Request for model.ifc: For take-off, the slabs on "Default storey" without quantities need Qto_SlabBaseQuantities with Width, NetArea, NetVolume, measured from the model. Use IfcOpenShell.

First a look at what the model holds.

```python
import ifcopenshell
import ifcopenshell.util.element
import ifcopenshell.util.unit

model = ifcopenshell.open("model.ifc")
print(model.schema)
for unit_type in ("LENGTHUNIT", "AREAUNIT", "VOLUMEUNIT"):
    print(unit_type, ifcopenshell.util.unit.calculate_unit_scale(model, unit_type))
storey = next(s for s in model.by_type("IfcBuildingStorey") if s.Name == "Default storey")
slabs = [e for e in ifcopenshell.util.element.get_decomposition(storey) if e.is_a("IfcSlab")]
for e in sorted(slabs, key=lambda e: e.id()):
    print(e.id(), e.is_a(), e.Name, list(ifcopenshell.util.element.get_psets(e, qtos_only=True)), sep=" | ")
```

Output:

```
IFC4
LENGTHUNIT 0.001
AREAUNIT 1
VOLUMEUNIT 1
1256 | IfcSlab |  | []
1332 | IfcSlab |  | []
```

```python
import ifcopenshell
import ifcopenshell.api.pset
import ifcopenshell.geom
import ifcopenshell.util.element
import ifcopenshell.util.shape
import ifcopenshell.util.unit

model = ifcopenshell.open("model.ifc")
unit_scale = ifcopenshell.util.unit.calculate_unit_scale(model)
area_scale = ifcopenshell.util.unit.calculate_unit_scale(model, "AREAUNIT")
volume_scale = ifcopenshell.util.unit.calculate_unit_scale(model, "VOLUMEUNIT")
settings = ifcopenshell.geom.settings()

storey = next(s for s in model.by_type("IfcBuildingStorey") if s.Name == "Default storey")
slabs = [e for e in ifcopenshell.util.element.get_decomposition(storey) if e.is_a("IfcSlab")]

for e in sorted(slabs, key=lambda e: e.id()):
    if ifcopenshell.util.element.get_psets(e, qtos_only=True, should_inherit=False):
        continue
    # Geometry comes back in metres, in the element's own axes.
    shape = ifcopenshell.geom.create_shape(settings, e)
    values = {
        "Width": ifcopenshell.util.shape.get_z(shape.geometry) / unit_scale,
        "NetArea": ifcopenshell.util.shape.get_footprint_area(shape.geometry) / area_scale,
        "NetVolume": ifcopenshell.util.shape.get_volume(shape.geometry) / volume_scale,
    }
    qto = ifcopenshell.api.pset.add_qto(model, product=e, name="Qto_SlabBaseQuantities")
    ifcopenshell.api.pset.edit_qto(model, qto=qto, properties=values)
    print(e.id(), {k: round(v, 3) for k, v in values.items()})

model.write("model_rev.ifc")
```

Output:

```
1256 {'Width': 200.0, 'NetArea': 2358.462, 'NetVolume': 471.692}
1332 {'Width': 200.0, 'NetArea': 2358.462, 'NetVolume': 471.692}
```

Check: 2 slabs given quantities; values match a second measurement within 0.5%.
